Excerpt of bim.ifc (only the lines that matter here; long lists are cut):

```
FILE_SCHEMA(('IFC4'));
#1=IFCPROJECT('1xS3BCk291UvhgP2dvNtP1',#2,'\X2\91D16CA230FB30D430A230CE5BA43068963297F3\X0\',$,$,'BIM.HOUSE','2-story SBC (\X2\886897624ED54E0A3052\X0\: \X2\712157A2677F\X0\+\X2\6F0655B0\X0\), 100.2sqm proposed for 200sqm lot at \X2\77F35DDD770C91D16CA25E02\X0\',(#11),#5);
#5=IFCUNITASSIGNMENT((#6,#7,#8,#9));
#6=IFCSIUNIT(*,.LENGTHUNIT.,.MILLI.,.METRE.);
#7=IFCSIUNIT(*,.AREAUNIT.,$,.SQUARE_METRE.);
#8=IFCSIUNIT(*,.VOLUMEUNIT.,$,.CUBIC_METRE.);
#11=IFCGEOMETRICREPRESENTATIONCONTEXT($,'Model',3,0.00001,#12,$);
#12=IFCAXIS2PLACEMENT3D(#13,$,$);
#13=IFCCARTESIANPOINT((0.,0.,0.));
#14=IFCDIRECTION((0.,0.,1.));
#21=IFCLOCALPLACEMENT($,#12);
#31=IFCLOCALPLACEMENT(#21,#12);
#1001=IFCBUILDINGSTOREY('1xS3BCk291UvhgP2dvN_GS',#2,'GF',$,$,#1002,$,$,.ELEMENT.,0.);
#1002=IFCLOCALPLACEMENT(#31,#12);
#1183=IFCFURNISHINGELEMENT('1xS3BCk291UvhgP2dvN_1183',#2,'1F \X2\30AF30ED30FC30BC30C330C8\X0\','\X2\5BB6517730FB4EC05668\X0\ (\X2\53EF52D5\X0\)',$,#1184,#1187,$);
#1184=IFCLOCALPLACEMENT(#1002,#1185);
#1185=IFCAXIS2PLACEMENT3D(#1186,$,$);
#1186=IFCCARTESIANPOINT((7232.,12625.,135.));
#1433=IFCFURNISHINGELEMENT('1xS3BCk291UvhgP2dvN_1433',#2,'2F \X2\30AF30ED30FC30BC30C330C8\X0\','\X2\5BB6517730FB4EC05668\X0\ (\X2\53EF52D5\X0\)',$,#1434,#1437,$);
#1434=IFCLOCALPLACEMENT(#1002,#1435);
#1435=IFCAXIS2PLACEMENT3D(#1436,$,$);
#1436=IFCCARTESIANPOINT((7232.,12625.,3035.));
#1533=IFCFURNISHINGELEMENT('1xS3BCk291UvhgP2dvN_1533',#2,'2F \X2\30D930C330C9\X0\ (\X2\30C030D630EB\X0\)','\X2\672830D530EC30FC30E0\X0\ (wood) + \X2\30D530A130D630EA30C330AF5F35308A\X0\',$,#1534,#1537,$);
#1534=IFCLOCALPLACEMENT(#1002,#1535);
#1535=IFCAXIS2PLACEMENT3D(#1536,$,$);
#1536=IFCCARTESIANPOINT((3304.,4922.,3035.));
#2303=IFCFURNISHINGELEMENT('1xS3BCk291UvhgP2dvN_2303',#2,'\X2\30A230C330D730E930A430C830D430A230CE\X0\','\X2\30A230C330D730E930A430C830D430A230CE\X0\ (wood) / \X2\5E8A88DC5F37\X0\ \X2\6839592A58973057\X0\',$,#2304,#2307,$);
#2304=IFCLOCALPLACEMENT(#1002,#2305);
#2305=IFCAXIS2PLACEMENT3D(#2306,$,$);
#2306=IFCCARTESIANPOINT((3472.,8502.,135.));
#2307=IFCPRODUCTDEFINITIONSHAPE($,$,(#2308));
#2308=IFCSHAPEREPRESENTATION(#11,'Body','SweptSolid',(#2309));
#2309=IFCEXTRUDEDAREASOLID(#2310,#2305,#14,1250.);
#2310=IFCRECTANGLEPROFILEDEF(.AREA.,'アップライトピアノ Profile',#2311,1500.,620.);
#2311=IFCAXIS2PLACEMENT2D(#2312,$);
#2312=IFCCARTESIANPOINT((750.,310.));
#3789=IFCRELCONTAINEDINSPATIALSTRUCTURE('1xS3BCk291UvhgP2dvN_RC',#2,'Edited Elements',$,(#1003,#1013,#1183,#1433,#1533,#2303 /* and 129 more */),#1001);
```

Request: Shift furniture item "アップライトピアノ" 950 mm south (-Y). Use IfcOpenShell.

```python
import ifcopenshell
import ifcopenshell.api.geometry
import ifcopenshell.util.placement

model = ifcopenshell.open("bim.ifc")

item = model.by_id(2303)
matrix = ifcopenshell.util.placement.get_local_placement(item.ObjectPlacement)
matrix[1, 3] -= 950.0
ifcopenshell.api.geometry.edit_object_placement(model, product=item, matrix=matrix, is_si=False)

print(ifcopenshell.util.placement.get_local_placement(item.ObjectPlacement).round(3) + 0.0)

model.write("bim_v2.ifc")
```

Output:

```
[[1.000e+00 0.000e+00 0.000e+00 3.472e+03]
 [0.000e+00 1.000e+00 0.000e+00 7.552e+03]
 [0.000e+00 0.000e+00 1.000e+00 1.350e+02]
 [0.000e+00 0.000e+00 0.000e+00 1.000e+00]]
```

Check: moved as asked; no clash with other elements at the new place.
